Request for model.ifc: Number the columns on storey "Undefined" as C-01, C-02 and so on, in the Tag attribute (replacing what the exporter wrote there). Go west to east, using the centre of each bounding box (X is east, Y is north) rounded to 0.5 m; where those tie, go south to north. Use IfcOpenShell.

First a look at what the model holds.

```python
import ifcopenshell
import ifcopenshell.util.element
import ifcopenshell.util.placement

model = ifcopenshell.open("model.ifc")
print(model.schema)
storey = next(s for s in model.by_type("IfcBuildingStorey") if s.Name == "Undefined")
columns = [e for e in ifcopenshell.util.element.get_decomposition(storey) if e.is_a("IfcColumn")]
for e in sorted(columns, key=lambda e: e.id()):
    origin = ifcopenshell.util.placement.get_local_placement(e.ObjectPlacement)[:3, 3]
    print(e.id(), e.Tag, e.Name, origin.round(2) + 0.0, sep=" | ")
```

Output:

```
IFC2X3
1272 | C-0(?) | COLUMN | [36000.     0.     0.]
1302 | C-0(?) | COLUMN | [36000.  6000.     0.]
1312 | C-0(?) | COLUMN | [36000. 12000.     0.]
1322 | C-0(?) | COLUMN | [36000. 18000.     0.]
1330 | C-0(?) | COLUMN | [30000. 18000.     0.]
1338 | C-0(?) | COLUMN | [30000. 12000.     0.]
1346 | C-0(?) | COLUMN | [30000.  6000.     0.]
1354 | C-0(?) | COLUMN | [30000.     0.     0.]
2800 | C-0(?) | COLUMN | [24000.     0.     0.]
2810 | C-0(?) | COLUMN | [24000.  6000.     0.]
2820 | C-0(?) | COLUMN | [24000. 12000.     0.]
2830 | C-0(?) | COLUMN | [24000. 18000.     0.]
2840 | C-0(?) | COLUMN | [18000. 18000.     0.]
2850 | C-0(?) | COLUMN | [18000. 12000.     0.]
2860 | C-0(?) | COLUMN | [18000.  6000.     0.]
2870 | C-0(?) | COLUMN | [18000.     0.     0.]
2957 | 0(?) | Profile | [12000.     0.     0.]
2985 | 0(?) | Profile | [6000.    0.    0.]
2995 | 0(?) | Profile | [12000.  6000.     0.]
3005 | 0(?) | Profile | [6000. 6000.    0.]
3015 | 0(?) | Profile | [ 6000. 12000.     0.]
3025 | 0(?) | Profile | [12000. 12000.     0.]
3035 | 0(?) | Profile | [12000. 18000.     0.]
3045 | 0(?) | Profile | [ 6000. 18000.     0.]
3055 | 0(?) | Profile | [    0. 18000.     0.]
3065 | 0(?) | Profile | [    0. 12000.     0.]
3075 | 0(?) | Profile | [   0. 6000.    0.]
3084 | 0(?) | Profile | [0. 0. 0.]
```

```python
import ifcopenshell
import ifcopenshell.geom
import ifcopenshell.util.element
import ifcopenshell.util.shape

model = ifcopenshell.open("model.ifc")
settings = ifcopenshell.geom.settings()
settings.set("use-world-coords", True)


def centre(element):
    shape = ifcopenshell.geom.create_shape(settings, element)
    return ifcopenshell.util.shape.get_bbox_centroid(shape.geometry)


storey = next(s for s in model.by_type("IfcBuildingStorey") if s.Name == "Undefined")
columns = [e for e in ifcopenshell.util.element.get_decomposition(storey) if e.is_a("IfcColumn")]

# Insertion points can sit at a corner or the storey origin, so sort by the geometry (in metres).
centres = {e: centre(e) for e in columns}
columns.sort(key=lambda e: (round(centres[e][0] / 0.5), centres[e][1]))

for i, e in enumerate(columns, start=1):
    number = f"C-{i:02d}"
    e.Tag = number
    print(e.id(), number)

model.write("model_rev.ifc")
```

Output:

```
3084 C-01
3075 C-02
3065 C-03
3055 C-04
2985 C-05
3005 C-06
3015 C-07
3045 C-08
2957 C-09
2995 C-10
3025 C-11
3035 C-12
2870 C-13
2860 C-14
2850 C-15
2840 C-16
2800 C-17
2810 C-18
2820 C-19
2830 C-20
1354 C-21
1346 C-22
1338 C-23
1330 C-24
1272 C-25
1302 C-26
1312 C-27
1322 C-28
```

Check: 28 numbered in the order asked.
